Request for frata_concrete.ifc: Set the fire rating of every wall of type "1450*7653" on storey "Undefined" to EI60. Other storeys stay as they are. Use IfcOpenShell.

First a look at what the model holds.

```python
import ifcopenshell
import ifcopenshell.util.element

model = ifcopenshell.open("frata_concrete.ifc")
print(model.schema)
storey = next(s for s in model.by_type("IfcBuildingStorey") if s.Name == "Undefined")
walls = [e for e in ifcopenshell.util.element.get_decomposition(storey) if e.is_a("IfcWall")]
seen = {}
for e in walls:
    element_type = ifcopenshell.util.element.get_type(e)
    key = (element_type.Name if element_type != e and element_type else None, ifcopenshell.util.element.get_pset(e, "Pset_WallCommon", "FireRating"))
    seen[key] = seen.get(key, 0) + 1
for (name, value), count in sorted(seen.items(), key=str):
    print(count, "x", name, "|", value)
```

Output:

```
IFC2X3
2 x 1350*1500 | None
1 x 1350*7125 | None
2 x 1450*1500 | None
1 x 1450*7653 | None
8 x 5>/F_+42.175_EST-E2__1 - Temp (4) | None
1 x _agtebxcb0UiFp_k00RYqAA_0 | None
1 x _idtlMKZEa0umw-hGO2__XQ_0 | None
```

```python
import ifcopenshell
import ifcopenshell.api.pset
import ifcopenshell.util.element

model = ifcopenshell.open("frata_concrete.ifc")

storey = next(s for s in model.by_type("IfcBuildingStorey") if s.Name == "Undefined")
walls = [e for e in ifcopenshell.util.element.get_decomposition(storey) if e.is_a("IfcWall")]

count = 0
for e in walls:
    element_type = ifcopenshell.util.element.get_type(e)
    if element_type in (None, e) or element_type.Name != "1450*7653":
        continue
    # add_pset returns the element's existing set when there is one.
    pset = ifcopenshell.api.pset.add_pset(model, product=e, name="Pset_WallCommon")
    ifcopenshell.api.pset.edit_pset(model, pset=pset, properties={"FireRating": "EI60"})
    count += 1

print(count, "walls updated")

model.write("frata_concrete_rev.ifc")
```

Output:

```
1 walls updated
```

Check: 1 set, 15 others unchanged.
